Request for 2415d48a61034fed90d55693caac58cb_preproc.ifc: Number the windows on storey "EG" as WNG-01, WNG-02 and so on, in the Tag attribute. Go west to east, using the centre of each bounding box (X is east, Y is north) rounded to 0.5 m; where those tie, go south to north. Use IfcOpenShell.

First a look at what the model holds.

```python
import ifcopenshell
import ifcopenshell.util.element
import ifcopenshell.util.placement

model = ifcopenshell.open("2415d48a61034fed90d55693caac58cb_preproc.ifc")
print(model.schema)
storey = next(s for s in model.by_type("IfcBuildingStorey") if s.Name == "EG")
windows = [e for e in ifcopenshell.util.element.get_decomposition(storey) if e.is_a("IfcWindow")]
for e in sorted(windows, key=lambda e: e.id()):
    origin = ifcopenshell.util.placement.get_local_placement(e.ObjectPlacement)[:3, 3]
    print(e.id(), e.Tag, e.Name, origin.round(2) + 0.0, sep=" | ")
```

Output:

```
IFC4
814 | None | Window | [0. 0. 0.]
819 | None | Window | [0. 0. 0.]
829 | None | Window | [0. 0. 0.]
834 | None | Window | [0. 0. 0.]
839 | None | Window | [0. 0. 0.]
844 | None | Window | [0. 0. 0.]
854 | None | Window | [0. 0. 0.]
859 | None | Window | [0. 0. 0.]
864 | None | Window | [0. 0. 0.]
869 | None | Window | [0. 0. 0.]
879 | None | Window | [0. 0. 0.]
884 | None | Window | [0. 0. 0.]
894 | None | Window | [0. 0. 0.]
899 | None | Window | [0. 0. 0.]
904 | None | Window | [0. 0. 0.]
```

```python
import ifcopenshell
import ifcopenshell.geom
import ifcopenshell.util.element
import ifcopenshell.util.shape

model = ifcopenshell.open("2415d48a61034fed90d55693caac58cb_preproc.ifc")
settings = ifcopenshell.geom.settings()
settings.set("use-world-coords", True)


def centre(element):
    shape = ifcopenshell.geom.create_shape(settings, element)
    return ifcopenshell.util.shape.get_bbox_centroid(shape.geometry)


storey = next(s for s in model.by_type("IfcBuildingStorey") if s.Name == "EG")
windows = [e for e in ifcopenshell.util.element.get_decomposition(storey) if e.is_a("IfcWindow")]

# Insertion points can sit at a corner or the storey origin, so sort by the geometry (in metres).
centres = {e: centre(e) for e in windows}
windows.sort(key=lambda e: (round(centres[e][0] / 0.5), centres[e][1]))

for i, e in enumerate(windows, start=1):
    number = f"WNG-{i:02d}"
    e.Tag = number
    print(e.id(), number)

model.write("2415d48a61034fed90d55693caac58cb_preproc-out.ifc")
```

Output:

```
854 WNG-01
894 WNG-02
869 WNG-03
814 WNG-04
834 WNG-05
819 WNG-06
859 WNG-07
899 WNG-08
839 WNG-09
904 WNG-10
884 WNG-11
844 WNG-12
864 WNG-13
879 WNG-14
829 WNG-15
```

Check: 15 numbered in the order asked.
